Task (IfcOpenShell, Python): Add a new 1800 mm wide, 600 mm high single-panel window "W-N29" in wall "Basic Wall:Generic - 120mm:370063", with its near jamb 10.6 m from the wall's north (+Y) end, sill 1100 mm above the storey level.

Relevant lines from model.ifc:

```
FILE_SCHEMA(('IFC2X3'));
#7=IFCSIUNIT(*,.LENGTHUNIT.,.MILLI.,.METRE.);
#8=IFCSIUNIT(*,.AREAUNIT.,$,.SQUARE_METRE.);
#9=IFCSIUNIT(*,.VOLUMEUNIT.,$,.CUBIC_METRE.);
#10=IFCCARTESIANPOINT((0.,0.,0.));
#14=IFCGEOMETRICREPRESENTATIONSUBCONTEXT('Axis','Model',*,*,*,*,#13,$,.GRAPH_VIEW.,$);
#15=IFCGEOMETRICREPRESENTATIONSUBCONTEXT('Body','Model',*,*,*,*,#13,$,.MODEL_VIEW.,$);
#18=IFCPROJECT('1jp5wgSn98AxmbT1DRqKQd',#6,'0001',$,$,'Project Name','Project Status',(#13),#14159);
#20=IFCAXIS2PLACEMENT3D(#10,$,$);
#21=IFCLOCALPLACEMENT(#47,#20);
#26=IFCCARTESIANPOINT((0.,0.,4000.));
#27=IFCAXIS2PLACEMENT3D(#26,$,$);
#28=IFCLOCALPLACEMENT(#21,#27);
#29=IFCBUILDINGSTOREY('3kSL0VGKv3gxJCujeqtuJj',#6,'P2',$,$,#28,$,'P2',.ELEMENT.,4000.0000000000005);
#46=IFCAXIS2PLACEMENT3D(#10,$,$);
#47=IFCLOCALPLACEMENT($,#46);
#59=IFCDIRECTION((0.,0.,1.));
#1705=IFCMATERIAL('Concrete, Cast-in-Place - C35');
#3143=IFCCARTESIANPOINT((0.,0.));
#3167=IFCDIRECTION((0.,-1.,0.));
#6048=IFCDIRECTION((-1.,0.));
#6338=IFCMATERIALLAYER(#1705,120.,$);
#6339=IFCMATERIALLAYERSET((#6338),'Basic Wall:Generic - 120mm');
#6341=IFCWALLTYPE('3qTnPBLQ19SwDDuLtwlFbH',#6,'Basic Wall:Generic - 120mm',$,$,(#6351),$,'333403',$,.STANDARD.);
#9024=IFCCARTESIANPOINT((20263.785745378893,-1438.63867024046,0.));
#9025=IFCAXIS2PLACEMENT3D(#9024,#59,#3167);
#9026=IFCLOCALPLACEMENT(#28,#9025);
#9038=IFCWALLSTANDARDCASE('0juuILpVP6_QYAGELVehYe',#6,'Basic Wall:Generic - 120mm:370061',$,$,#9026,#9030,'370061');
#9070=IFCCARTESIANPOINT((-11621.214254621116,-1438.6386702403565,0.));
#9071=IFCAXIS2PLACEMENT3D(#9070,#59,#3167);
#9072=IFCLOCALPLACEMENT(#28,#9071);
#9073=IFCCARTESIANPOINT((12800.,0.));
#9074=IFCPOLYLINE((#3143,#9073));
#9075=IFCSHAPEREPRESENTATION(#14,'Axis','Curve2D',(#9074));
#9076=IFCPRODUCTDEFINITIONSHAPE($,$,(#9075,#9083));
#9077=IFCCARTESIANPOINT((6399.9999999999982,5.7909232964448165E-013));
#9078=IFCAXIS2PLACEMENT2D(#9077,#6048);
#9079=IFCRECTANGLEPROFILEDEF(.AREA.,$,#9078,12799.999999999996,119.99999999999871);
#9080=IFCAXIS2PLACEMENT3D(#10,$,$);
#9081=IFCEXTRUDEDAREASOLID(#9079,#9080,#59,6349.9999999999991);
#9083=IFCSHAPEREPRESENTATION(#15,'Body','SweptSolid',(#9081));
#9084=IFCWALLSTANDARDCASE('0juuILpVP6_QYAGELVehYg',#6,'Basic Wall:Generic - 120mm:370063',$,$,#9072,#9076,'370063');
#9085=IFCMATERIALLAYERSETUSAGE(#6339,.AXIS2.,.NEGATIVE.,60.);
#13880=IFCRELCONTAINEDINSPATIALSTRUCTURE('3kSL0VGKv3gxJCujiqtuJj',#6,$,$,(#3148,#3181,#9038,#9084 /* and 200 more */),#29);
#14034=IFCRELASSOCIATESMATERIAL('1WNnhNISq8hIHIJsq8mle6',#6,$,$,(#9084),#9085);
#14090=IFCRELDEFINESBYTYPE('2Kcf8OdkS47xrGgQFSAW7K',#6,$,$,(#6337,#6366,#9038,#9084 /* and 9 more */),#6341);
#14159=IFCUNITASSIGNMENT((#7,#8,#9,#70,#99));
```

```python
import numpy as np
import ifcopenshell
import ifcopenshell.api.feature
import ifcopenshell.api.geometry
import ifcopenshell.api.root
import ifcopenshell.api.spatial
import ifcopenshell.api.type
import ifcopenshell.geom
import ifcopenshell.util.element
import ifcopenshell.util.placement
import ifcopenshell.util.representation
import ifcopenshell.util.shape
import ifcopenshell.util.unit

model = ifcopenshell.open("model.ifc")
unit_scale = ifcopenshell.util.unit.calculate_unit_scale(model)
settings = ifcopenshell.geom.settings()


def volume(element):
    """Net volume in cubic metres, openings subtracted."""
    shape = ifcopenshell.geom.create_shape(settings, element)
    return ifcopenshell.util.shape.get_volume(shape.geometry)


wall = model.by_guid("0juuILpVP6_QYAGELVehYg")
storey = ifcopenshell.util.element.get_container(wall, ifc_class="IfcBuildingStorey")
context = ifcopenshell.util.representation.get_context(model, "Model", "Body", "MODEL_VIEW")
before = volume(wall)

width, height, from_end, sill = 1.8, 0.6, 10.6, 1.1  # metres

# The wall runs along its own X axis, and the end named is its -X end.
wall_shape = ifcopenshell.geom.create_shape(settings, wall)
x, y, z = ifcopenshell.util.shape.get_vertices(wall_shape.geometry).T
start = x.min() + from_end
face, thickness = float(y.min()), float(y.max() - y.min())
wall_matrix = ifcopenshell.util.placement.get_local_placement(wall.ObjectPlacement)
level = ifcopenshell.util.placement.get_local_placement(storey.ObjectPlacement)[2, 3]


def in_wall(x, y):
    """Placement at x, y metres in the wall's axes, at sill height."""
    matrix = wall_matrix.copy()
    matrix[:, 3] = wall_matrix @ np.array([x / unit_scale, y / unit_scale, 0.0, 1.0])
    matrix[2, 3] = level + sill / unit_scale
    return matrix


# Opening: a box that overshoots both wall faces by 50 mm.
opening = ifcopenshell.api.root.create_entity(model, ifc_class="IfcOpeningElement")
box = ifcopenshell.api.geometry.add_wall_representation(
    model, context=context, length=width, height=height, thickness=thickness + 0.1
)
ifcopenshell.api.geometry.assign_representation(model, product=opening, representation=box)
ifcopenshell.api.geometry.edit_object_placement(model, product=opening, matrix=in_wall(start, face - 0.05), is_si=False)
ifcopenshell.api.feature.add_feature(model, feature=opening, element=wall)

window = ifcopenshell.api.root.create_entity(model, ifc_class="IfcWindow", name="W-N29")
window.OverallWidth, window.OverallHeight = width / unit_scale, height / unit_scale
body = ifcopenshell.api.geometry.add_window_representation(
    model,
    context=context,
    overall_width=window.OverallWidth,
    overall_height=window.OverallHeight,
    partition_type="SINGLE_PANEL",
)
ifcopenshell.api.geometry.assign_representation(model, product=window, representation=body)
ifcopenshell.api.spatial.assign_container(model, products=[window], relating_structure=storey)
fills = ifcopenshell.api.feature.add_filling(model, opening=opening, element=window)
fills.OwnerHistory = window.OwnerHistory  # required in IFC2X3

# IFC2X3 keeps the operation on the window style.
style = ifcopenshell.api.root.create_entity(model, ifc_class="IfcWindowStyle", name="W-N29")
style.OperationType, style.ConstructionType = "SINGLE_PANEL", "NOTDEFINED"
style.ParameterTakesPrecedence = style.Sizeable = False
ifcopenshell.api.type.assign_type(model, related_objects=[window], relating_type=style)

# Centre the window in the wall's thickness.
ifcopenshell.api.geometry.edit_object_placement(model, product=window, matrix=in_wall(start, face), is_si=False)
window_shape = ifcopenshell.geom.create_shape(settings, window)
depth = ifcopenshell.util.shape.get_vertices(window_shape.geometry)[:, 1]
offset = face + thickness / 2 - (depth.min() + depth.max()) / 2
ifcopenshell.api.geometry.edit_object_placement(model, product=window, matrix=in_wall(start, offset), is_si=False)

after = volume(wall)

print(f"wall volume {before:.3f} -> {after:.3f} m3")

model.write("model_rev.ifc")
```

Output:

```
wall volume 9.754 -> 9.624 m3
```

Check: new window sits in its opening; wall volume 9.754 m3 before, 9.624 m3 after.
